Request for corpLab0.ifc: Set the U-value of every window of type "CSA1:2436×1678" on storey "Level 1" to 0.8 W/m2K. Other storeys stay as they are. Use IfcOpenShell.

First a look at what the model holds.

```python
import ifcopenshell
import ifcopenshell.util.element

model = ifcopenshell.open("corpLab0.ifc")
print(model.schema)
storey = next(s for s in model.by_type("IfcBuildingStorey") if s.Name == "Level 1")
windows = [e for e in ifcopenshell.util.element.get_decomposition(storey) if e.is_a("IfcWindow")]
seen = {}
for e in windows:
    element_type = ifcopenshell.util.element.get_type(e)
    key = (element_type.Name if element_type != e and element_type else None, ifcopenshell.util.element.get_pset(e, "Pset_WindowCommon", "ThermalTransmittance"))
    seen[key] = seen.get(key, 0) + 1
for (name, value), count in sorted(seen.items(), key=str):
    print(count, "x", name, "|", value)
```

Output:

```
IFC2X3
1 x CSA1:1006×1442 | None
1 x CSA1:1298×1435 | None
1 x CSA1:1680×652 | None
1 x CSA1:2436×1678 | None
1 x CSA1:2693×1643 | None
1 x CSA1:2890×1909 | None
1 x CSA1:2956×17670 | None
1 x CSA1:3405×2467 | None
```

```python
import ifcopenshell
import ifcopenshell.api.pset
import ifcopenshell.util.element

model = ifcopenshell.open("corpLab0.ifc")

storey = next(s for s in model.by_type("IfcBuildingStorey") if s.Name == "Level 1")
windows = [e for e in ifcopenshell.util.element.get_decomposition(storey) if e.is_a("IfcWindow")]

count = 0
for e in windows:
    element_type = ifcopenshell.util.element.get_type(e)
    if element_type in (None, e) or element_type.Name != "CSA1:2436×1678":
        continue
    # add_pset returns the element's existing set when there is one.
    pset = ifcopenshell.api.pset.add_pset(model, product=e, name="Pset_WindowCommon")
    ifcopenshell.api.pset.edit_pset(model, pset=pset, properties={"ThermalTransmittance": 0.8})
    count += 1

print(count, "windows updated")

model.write("corpLab0_rev.ifc")
```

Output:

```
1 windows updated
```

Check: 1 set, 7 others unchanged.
